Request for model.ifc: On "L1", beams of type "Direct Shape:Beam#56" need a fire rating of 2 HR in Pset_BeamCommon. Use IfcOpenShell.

First a look at what the model holds.

```python
import ifcopenshell
import ifcopenshell.util.element

model = ifcopenshell.open("model.ifc")
print(model.schema)
storey = next(s for s in model.by_type("IfcBuildingStorey") if s.Name == "L1")
beams = [e for e in ifcopenshell.util.element.get_decomposition(storey) if e.is_a("IfcBeam")]
seen = {}
for e in beams:
    element_type = ifcopenshell.util.element.get_type(e)
    key = (element_type.Name if element_type != e and element_type else None, ifcopenshell.util.element.get_pset(e, "Pset_BeamCommon", "FireRating"))
    seen[key] = seen.get(key, 0) + 1
for (name, value), count in sorted(seen.items(), key=str):
    print(count, "x", name, "|", value)
```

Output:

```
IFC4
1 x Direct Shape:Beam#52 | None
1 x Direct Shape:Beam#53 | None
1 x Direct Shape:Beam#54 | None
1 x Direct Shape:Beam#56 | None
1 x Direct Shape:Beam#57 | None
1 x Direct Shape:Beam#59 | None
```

```python
import ifcopenshell
import ifcopenshell.api.pset
import ifcopenshell.util.element

model = ifcopenshell.open("model.ifc")

storey = next(s for s in model.by_type("IfcBuildingStorey") if s.Name == "L1")
beams = [e for e in ifcopenshell.util.element.get_decomposition(storey) if e.is_a("IfcBeam")]

count = 0
for e in beams:
    element_type = ifcopenshell.util.element.get_type(e)
    if element_type in (None, e) or element_type.Name != "Direct Shape:Beam#56":
        continue
    # add_pset returns the element's existing set when there is one.
    pset = ifcopenshell.api.pset.add_pset(model, product=e, name="Pset_BeamCommon")
    ifcopenshell.api.pset.edit_pset(model, pset=pset, properties={"FireRating": "2 HR"})
    count += 1

print(count, "beams updated")

model.write("model_v2.ifc")
```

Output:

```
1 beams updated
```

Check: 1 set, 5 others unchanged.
